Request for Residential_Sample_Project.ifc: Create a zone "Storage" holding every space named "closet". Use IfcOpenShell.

First a look at what the model holds.

```python
import ifcopenshell

model = ifcopenshell.open("Residential_Sample_Project.ifc")
print(model.schema)
seen = {}
for space in model.by_type("IfcSpace"):
    seen[space.LongName] = seen.get(space.LongName, 0) + 1
for name, count in sorted(seen.items(), key=str):
    print(count, "x", name)
print("zones:", [z.Name for z in model.by_type("IfcZone")][:20])
```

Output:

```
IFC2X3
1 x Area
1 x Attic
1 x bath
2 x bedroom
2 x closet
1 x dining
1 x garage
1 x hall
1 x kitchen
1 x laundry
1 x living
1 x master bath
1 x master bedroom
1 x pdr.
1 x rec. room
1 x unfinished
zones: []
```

```python
import ifcopenshell
import ifcopenshell.api.group
import ifcopenshell.api.root

model = ifcopenshell.open("Residential_Sample_Project.ifc")

names = {"closet"}
spaces = [s for s in model.by_type("IfcSpace") if s.LongName in names]

zone = ifcopenshell.api.root.create_entity(model, ifc_class="IfcZone", name="Storage")
ifcopenshell.api.group.assign_group(model, products=spaces, group=zone)
print(len(spaces), "spaces in", zone.Name)

model.write("Residential_Sample_Project_updated.ifc")
```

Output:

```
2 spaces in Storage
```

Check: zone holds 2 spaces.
